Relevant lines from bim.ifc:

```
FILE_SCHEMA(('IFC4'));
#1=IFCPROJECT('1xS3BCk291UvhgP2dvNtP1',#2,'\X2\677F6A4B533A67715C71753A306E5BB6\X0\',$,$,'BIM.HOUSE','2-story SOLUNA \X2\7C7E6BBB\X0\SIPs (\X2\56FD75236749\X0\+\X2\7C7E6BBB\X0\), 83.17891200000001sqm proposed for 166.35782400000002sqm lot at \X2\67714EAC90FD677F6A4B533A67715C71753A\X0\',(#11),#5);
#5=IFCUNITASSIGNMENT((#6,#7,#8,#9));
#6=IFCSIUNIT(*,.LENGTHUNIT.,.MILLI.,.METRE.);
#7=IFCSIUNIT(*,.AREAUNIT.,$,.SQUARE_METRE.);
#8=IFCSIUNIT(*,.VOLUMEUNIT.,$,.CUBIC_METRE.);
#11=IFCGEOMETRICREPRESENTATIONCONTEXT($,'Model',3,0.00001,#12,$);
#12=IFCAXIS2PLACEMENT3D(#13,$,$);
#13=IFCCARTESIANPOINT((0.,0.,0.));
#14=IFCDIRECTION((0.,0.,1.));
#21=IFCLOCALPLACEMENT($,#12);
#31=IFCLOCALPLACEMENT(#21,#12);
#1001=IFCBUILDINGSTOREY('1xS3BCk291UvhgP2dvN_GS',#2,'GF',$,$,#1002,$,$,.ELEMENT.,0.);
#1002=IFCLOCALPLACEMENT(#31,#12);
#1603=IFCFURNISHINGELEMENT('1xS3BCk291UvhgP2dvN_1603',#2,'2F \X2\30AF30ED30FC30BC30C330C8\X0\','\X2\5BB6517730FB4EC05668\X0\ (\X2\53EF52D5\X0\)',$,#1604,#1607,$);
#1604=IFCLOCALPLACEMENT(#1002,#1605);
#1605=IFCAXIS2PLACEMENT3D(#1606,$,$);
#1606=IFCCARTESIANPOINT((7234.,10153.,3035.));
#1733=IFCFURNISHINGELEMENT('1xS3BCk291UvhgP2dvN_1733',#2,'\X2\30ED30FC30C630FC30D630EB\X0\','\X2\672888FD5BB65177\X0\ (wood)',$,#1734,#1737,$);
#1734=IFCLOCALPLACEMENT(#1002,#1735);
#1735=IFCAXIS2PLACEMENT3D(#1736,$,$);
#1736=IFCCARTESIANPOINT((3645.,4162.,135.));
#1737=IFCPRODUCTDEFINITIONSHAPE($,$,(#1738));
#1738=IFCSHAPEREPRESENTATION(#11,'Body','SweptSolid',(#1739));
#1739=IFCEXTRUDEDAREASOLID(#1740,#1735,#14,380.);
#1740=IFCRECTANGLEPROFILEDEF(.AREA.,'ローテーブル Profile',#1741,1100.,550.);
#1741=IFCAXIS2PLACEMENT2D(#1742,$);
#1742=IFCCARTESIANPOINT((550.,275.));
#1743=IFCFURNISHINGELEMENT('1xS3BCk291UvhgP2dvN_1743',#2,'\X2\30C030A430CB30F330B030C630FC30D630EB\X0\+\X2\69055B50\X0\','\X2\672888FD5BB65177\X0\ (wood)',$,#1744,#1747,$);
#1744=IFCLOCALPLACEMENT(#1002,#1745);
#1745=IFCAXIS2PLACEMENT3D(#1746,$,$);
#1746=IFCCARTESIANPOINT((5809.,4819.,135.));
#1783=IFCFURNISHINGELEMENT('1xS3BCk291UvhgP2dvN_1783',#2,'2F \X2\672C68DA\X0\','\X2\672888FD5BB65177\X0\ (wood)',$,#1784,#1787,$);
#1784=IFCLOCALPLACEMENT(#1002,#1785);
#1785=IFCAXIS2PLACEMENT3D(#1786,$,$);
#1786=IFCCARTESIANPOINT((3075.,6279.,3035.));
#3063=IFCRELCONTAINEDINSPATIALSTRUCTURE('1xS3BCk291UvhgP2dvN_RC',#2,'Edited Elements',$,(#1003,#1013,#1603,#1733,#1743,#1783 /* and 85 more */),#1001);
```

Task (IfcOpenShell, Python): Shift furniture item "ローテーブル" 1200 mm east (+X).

```python
import ifcopenshell
import ifcopenshell.api.geometry
import ifcopenshell.util.placement
import ifcopenshell.util.unit

model = ifcopenshell.open("bim.ifc")
unit_scale = ifcopenshell.util.unit.calculate_unit_scale(model)

item = model.by_guid("1xS3BCk291UvhgP2dvN_1733")
matrix = ifcopenshell.util.placement.get_local_placement(item.ObjectPlacement)
matrix[0, 3] += 1.2 / unit_scale
ifcopenshell.api.geometry.edit_object_placement(model, product=item, matrix=matrix, is_si=False)

print(ifcopenshell.util.placement.get_local_placement(item.ObjectPlacement).round(3) + 0.0)

model.write("bim-out.ifc")
```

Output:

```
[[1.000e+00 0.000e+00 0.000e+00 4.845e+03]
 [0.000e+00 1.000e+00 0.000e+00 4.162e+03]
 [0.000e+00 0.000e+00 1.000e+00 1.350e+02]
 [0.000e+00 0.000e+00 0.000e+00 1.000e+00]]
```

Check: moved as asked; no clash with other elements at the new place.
